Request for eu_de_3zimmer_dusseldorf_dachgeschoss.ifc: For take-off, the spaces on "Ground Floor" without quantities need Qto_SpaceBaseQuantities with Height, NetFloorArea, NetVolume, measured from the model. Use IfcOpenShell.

First a look at what the model holds.

```python
import ifcopenshell
import ifcopenshell.util.element
import ifcopenshell.util.unit

model = ifcopenshell.open("eu_de_3zimmer_dusseldorf_dachgeschoss.ifc")
print(model.schema)
for unit_type in ("LENGTHUNIT", "AREAUNIT", "VOLUMEUNIT"):
    print(unit_type, ifcopenshell.util.unit.calculate_unit_scale(model, unit_type))
storey = next(s for s in model.by_type("IfcBuildingStorey") if s.Name == "Ground Floor")
spaces = [e for e in ifcopenshell.util.element.get_decomposition(storey) if e.is_a("IfcSpace")]
for e in sorted(spaces, key=lambda e: e.id()):
    print(e.id(), e.is_a(), e.Name, list(ifcopenshell.util.element.get_psets(e, qtos_only=True)), sep=" | ")
```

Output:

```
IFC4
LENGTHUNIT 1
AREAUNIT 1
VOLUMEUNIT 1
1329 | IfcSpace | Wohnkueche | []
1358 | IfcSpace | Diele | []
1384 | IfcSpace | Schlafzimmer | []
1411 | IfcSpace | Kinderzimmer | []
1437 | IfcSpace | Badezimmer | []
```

```python
import ifcopenshell
import ifcopenshell.api.pset
import ifcopenshell.geom
import ifcopenshell.util.element
import ifcopenshell.util.shape
import ifcopenshell.util.unit

model = ifcopenshell.open("eu_de_3zimmer_dusseldorf_dachgeschoss.ifc")
unit_scale = ifcopenshell.util.unit.calculate_unit_scale(model)
area_scale = ifcopenshell.util.unit.calculate_unit_scale(model, "AREAUNIT")
volume_scale = ifcopenshell.util.unit.calculate_unit_scale(model, "VOLUMEUNIT")
settings = ifcopenshell.geom.settings()

storey = next(s for s in model.by_type("IfcBuildingStorey") if s.Name == "Ground Floor")
spaces = [e for e in ifcopenshell.util.element.get_decomposition(storey) if e.is_a("IfcSpace")]

for e in sorted(spaces, key=lambda e: e.id()):
    if ifcopenshell.util.element.get_psets(e, qtos_only=True, should_inherit=False):
        continue
    # Geometry comes back in metres, in the element's own axes.
    shape = ifcopenshell.geom.create_shape(settings, e)
    values = {
        "Height": ifcopenshell.util.shape.get_z(shape.geometry) / unit_scale,
        "NetFloorArea": ifcopenshell.util.shape.get_footprint_area(shape.geometry) / area_scale,
        "NetVolume": ifcopenshell.util.shape.get_volume(shape.geometry) / volume_scale,
    }
    qto = ifcopenshell.api.pset.add_qto(model, product=e, name="Qto_SpaceBaseQuantities")
    ifcopenshell.api.pset.edit_qto(model, qto=qto, properties=values)
    print(e.id(), {k: round(v, 3) for k, v in values.items()})

model.write("eu_de_3zimmer_dusseldorf_dachgeschoss_v2.ifc")
```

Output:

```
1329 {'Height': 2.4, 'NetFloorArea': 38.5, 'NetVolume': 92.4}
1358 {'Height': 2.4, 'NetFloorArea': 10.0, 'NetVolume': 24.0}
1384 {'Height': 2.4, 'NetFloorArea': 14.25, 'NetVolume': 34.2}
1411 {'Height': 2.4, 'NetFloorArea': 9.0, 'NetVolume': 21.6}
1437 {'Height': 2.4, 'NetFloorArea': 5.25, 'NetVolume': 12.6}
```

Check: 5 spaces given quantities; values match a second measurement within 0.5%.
